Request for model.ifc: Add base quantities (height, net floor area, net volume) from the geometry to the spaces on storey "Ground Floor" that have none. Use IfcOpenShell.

First a look at what the model holds.

```python
import ifcopenshell
import ifcopenshell.util.element
import ifcopenshell.util.unit

model = ifcopenshell.open("model.ifc")
print(model.schema)
for unit_type in ("LENGTHUNIT", "AREAUNIT", "VOLUMEUNIT"):
    print(unit_type, ifcopenshell.util.unit.calculate_unit_scale(model, unit_type))
storey = next(s for s in model.by_type("IfcBuildingStorey") if s.Name == "Ground Floor")
spaces = [e for e in ifcopenshell.util.element.get_decomposition(storey) if e.is_a("IfcSpace")]
for e in sorted(spaces, key=lambda e: e.id()):
    print(e.id(), e.is_a(), e.Name, list(ifcopenshell.util.element.get_psets(e, qtos_only=True)), sep=" | ")
```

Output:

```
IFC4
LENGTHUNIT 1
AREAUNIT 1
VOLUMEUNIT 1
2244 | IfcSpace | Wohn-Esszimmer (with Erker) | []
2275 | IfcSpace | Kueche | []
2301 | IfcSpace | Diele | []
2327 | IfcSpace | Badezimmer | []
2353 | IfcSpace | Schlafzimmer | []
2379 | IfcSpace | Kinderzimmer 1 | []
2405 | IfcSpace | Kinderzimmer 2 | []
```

```python
import ifcopenshell
import ifcopenshell.api.pset
import ifcopenshell.geom
import ifcopenshell.util.element
import ifcopenshell.util.shape
import ifcopenshell.util.unit

model = ifcopenshell.open("model.ifc")
unit_scale = ifcopenshell.util.unit.calculate_unit_scale(model)
area_scale = ifcopenshell.util.unit.calculate_unit_scale(model, "AREAUNIT")
volume_scale = ifcopenshell.util.unit.calculate_unit_scale(model, "VOLUMEUNIT")
settings = ifcopenshell.geom.settings()

storey = next(s for s in model.by_type("IfcBuildingStorey") if s.Name == "Ground Floor")
spaces = [e for e in ifcopenshell.util.element.get_decomposition(storey) if e.is_a("IfcSpace")]

for e in sorted(spaces, key=lambda e: e.id()):
    if ifcopenshell.util.element.get_psets(e, qtos_only=True, should_inherit=False):
        continue
    # Geometry comes back in metres, in the element's own axes.
    shape = ifcopenshell.geom.create_shape(settings, e)
    values = {
        "Height": ifcopenshell.util.shape.get_z(shape.geometry) / unit_scale,
        "NetFloorArea": ifcopenshell.util.shape.get_footprint_area(shape.geometry) / area_scale,
        "NetVolume": ifcopenshell.util.shape.get_volume(shape.geometry) / volume_scale,
    }
    qto = ifcopenshell.api.pset.add_qto(model, product=e, name="Qto_SpaceBaseQuantities")
    ifcopenshell.api.pset.edit_qto(model, qto=qto, properties=values)
    print(e.id(), {k: round(v, 3) for k, v in values.items()})

model.write("model_updated.ifc")
```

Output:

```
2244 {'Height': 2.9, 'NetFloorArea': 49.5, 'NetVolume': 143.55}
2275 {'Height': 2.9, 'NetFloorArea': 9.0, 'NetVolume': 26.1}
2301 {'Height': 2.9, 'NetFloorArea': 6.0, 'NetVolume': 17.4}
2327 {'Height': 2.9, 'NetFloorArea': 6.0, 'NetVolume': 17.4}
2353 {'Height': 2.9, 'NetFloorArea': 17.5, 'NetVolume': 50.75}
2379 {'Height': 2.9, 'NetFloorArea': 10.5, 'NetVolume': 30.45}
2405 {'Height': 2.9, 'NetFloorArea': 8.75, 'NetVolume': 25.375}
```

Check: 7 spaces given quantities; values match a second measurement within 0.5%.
